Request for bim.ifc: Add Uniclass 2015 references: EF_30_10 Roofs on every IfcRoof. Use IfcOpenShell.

First a look at what the model holds.

```python
import ifcopenshell

model = ifcopenshell.open("bim.ifc")
print(model.schema)
print("classifications:", [c.Name for c in model.by_type("IfcClassification")])
for ifc_class in ("IfcDoor", "IfcRoof", "IfcStair", "IfcWall", "IfcWindow"):
    print(ifc_class, len(model.by_type(ifc_class)))
```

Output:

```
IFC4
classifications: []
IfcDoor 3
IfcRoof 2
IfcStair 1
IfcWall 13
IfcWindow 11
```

```python
import ifcopenshell
import ifcopenshell.api.classification

model = ifcopenshell.open("bim.ifc")

system = ifcopenshell.api.classification.add_classification(model, classification="Uniclass 2015")

codes = {
    "IfcRoof": ("EF_30_10", "Roofs"),
}
for ifc_class, (code, name) in codes.items():
    products = model.by_type(ifc_class)
    ifcopenshell.api.classification.add_reference(
        model, products=products, classification=system, identification=code, name=name
    )
    print(code, len(products))

model.write("bim_v2.ifc")
```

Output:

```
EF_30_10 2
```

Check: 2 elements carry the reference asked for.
